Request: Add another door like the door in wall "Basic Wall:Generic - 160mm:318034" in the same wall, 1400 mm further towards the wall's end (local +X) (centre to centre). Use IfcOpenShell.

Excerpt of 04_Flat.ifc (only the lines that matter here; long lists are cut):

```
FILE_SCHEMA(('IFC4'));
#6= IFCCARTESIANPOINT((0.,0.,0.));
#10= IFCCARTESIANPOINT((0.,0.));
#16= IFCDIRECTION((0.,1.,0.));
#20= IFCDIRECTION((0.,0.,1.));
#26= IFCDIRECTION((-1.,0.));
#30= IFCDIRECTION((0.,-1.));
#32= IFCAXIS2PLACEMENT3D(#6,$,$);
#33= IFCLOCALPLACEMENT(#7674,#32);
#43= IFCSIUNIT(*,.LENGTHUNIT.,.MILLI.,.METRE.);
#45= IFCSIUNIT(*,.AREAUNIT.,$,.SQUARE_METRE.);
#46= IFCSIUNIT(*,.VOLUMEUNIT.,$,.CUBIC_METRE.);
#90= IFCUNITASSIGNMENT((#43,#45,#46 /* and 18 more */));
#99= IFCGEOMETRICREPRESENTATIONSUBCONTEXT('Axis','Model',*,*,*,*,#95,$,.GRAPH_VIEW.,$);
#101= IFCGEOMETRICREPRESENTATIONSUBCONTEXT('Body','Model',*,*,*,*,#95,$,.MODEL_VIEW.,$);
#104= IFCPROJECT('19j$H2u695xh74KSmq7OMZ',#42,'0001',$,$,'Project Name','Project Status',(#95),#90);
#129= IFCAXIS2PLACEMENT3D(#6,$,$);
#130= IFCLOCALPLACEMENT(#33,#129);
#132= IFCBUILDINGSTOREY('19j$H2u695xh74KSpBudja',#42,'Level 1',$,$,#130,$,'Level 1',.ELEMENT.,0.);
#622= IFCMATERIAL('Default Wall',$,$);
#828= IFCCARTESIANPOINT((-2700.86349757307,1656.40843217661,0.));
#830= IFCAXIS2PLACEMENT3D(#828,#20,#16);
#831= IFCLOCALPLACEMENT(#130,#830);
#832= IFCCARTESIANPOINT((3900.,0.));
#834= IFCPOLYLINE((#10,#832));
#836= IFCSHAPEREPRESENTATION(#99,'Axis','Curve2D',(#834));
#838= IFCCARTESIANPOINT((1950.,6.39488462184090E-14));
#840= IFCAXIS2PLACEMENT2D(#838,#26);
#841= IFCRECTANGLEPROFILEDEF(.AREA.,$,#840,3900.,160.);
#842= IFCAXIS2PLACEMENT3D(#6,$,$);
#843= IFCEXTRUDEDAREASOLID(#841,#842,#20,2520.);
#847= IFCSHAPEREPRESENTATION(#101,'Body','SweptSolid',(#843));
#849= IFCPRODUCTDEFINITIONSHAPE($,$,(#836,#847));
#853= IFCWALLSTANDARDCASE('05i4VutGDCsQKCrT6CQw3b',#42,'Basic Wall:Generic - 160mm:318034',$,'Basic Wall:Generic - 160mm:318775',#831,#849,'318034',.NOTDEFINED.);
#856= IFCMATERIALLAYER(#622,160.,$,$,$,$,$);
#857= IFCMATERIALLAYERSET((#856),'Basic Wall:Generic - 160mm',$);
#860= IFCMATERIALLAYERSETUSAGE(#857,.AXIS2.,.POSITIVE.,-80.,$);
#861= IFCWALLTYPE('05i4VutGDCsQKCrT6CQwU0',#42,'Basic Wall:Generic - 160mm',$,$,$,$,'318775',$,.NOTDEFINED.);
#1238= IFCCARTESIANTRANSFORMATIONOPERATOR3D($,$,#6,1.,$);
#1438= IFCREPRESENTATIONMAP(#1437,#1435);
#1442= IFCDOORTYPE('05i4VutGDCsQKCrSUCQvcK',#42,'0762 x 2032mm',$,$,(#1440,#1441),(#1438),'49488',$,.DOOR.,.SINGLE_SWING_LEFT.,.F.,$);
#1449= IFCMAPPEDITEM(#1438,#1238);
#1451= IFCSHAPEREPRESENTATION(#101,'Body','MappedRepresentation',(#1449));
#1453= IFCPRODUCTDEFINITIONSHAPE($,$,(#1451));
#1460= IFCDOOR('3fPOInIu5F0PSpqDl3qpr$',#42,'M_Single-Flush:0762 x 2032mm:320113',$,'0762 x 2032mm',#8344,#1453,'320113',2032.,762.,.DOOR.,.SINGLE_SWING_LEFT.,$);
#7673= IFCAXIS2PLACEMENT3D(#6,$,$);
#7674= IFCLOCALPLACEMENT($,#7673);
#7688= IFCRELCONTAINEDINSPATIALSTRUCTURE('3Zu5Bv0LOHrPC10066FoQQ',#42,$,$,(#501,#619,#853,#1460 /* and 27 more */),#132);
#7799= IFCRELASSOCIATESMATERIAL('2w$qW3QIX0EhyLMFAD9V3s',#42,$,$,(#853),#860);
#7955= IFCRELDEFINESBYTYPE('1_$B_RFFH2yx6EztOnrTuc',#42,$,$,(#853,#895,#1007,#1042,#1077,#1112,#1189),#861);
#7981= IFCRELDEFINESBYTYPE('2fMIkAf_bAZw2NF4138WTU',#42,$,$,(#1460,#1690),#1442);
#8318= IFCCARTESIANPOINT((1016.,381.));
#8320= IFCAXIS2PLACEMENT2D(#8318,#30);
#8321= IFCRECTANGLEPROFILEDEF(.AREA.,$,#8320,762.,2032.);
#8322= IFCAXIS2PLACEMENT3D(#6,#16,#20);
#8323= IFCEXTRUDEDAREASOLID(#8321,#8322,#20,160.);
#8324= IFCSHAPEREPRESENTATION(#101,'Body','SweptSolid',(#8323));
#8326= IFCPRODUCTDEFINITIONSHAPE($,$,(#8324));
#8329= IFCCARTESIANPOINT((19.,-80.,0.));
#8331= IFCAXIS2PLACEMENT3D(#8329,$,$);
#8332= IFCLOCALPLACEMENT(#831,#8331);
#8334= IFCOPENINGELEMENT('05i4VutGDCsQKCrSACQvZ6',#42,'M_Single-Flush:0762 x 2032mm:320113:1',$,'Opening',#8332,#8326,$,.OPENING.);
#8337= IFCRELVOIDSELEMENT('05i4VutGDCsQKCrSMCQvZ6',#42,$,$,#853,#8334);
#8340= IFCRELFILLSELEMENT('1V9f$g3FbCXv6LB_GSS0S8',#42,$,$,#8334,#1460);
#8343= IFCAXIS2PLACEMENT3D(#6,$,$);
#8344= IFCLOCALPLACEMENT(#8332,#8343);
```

```python
import ifcopenshell
import ifcopenshell.api.feature
import ifcopenshell.api.geometry
import ifcopenshell.api.root
import ifcopenshell.geom
import ifcopenshell.util.element
import ifcopenshell.util.placement
import ifcopenshell.util.shape

model = ifcopenshell.open("04_Flat.ifc")
settings = ifcopenshell.geom.settings()


def volume(element):
    """Net volume in cubic metres, openings subtracted."""
    shape = ifcopenshell.geom.create_shape(settings, element)
    return ifcopenshell.util.shape.get_volume(shape.geometry)


def reuse_history(source, copy):
    """copy_class also copies each property set's owner history, people and application; keep the originals."""
    for rel in copy.IsDefinedBy:
        if rel.is_a("IfcRelDefinesByProperties") and (history := rel.RelatingPropertyDefinition.OwnerHistory):
            rel.RelatingPropertyDefinition.OwnerHistory = source.OwnerHistory
            ifcopenshell.util.element.remove_deep2(model, history)


door = model.by_guid("3fPOInIu5F0PSpqDl3qpr$")
opening = door.FillsVoids[0].RelatingOpeningElement
wall = opening.VoidsElements[0].RelatingBuildingElement
before = volume(wall)
shift = ifcopenshell.util.placement.get_local_placement(wall.ObjectPlacement)[:3, 0] * 1400.0

# copy_class copies the void relationship, type, container and properties, but no geometry.
new_opening = ifcopenshell.api.root.copy_class(model, product=opening)
new_opening.Representation = ifcopenshell.util.element.copy_deep(
    model, opening.Representation, exclude=["IfcGeometricRepresentationContext", "IfcRepresentationMap"]
)
new_opening.Name = "M_Single-Flush:0762 x 2032mm"
new_door = ifcopenshell.api.root.copy_class(model, product=door)
new_door.Representation = ifcopenshell.util.element.copy_deep(
    model, door.Representation, exclude=["IfcGeometricRepresentationContext", "IfcRepresentationMap"]
)
new_door.Name = "M_Single-Flush:0762 x 2032mm"
new_door.Tag = None
reuse_history(door, new_door)
ifcopenshell.api.feature.add_filling(model, opening=new_opening, element=new_door)

for old, new in ((opening, new_opening), (door, new_door)):
    matrix = ifcopenshell.util.placement.get_local_placement(old.ObjectPlacement)
    matrix[:3, 3] += shift
    ifcopenshell.api.geometry.edit_object_placement(model, product=new, matrix=matrix, is_si=False)

after = volume(wall)

print(f"wall volume {before:.3f} -> {after:.3f} m3")

model.write("04_Flat-out.ifc")
```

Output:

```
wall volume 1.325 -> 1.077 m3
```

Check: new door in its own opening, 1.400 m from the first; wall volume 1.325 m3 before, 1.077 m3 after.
